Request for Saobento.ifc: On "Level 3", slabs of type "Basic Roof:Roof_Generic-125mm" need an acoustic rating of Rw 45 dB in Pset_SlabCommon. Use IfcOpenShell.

First a look at what the model holds.

```python
import ifcopenshell
import ifcopenshell.util.element

model = ifcopenshell.open("Saobento.ifc")
print(model.schema)
storey = next(s for s in model.by_type("IfcBuildingStorey") if s.Name == "Level 3")
slabs = [e for e in ifcopenshell.util.element.get_decomposition(storey) if e.is_a("IfcSlab")]
seen = {}
for e in slabs:
    element_type = ifcopenshell.util.element.get_type(e)
    key = (element_type.Name if element_type != e and element_type else None, ifcopenshell.util.element.get_pset(e, "Pset_SlabCommon", "AcousticRating"))
    seen[key] = seen.get(key, 0) + 1
for (name, value), count in sorted(seen.items(), key=str):
    print(count, "x", name, "|", value)
```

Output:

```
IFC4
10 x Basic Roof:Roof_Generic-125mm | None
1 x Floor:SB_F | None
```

```python
import ifcopenshell
import ifcopenshell.api.pset
import ifcopenshell.util.element

model = ifcopenshell.open("Saobento.ifc")

storey = next(s for s in model.by_type("IfcBuildingStorey") if s.Name == "Level 3")
slabs = [e for e in ifcopenshell.util.element.get_decomposition(storey) if e.is_a("IfcSlab")]

count = 0
for e in slabs:
    element_type = ifcopenshell.util.element.get_type(e)
    if element_type in (None, e) or element_type.Name != "Basic Roof:Roof_Generic-125mm":
        continue
    # add_pset returns the element's existing set when there is one.
    pset = ifcopenshell.api.pset.add_pset(model, product=e, name="Pset_SlabCommon")
    ifcopenshell.api.pset.edit_pset(model, pset=pset, properties={"AcousticRating": "Rw 45 dB"})
    count += 1

print(count, "slabs updated")

model.write("Saobento-out.ifc")
```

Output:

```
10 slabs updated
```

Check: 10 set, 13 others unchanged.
